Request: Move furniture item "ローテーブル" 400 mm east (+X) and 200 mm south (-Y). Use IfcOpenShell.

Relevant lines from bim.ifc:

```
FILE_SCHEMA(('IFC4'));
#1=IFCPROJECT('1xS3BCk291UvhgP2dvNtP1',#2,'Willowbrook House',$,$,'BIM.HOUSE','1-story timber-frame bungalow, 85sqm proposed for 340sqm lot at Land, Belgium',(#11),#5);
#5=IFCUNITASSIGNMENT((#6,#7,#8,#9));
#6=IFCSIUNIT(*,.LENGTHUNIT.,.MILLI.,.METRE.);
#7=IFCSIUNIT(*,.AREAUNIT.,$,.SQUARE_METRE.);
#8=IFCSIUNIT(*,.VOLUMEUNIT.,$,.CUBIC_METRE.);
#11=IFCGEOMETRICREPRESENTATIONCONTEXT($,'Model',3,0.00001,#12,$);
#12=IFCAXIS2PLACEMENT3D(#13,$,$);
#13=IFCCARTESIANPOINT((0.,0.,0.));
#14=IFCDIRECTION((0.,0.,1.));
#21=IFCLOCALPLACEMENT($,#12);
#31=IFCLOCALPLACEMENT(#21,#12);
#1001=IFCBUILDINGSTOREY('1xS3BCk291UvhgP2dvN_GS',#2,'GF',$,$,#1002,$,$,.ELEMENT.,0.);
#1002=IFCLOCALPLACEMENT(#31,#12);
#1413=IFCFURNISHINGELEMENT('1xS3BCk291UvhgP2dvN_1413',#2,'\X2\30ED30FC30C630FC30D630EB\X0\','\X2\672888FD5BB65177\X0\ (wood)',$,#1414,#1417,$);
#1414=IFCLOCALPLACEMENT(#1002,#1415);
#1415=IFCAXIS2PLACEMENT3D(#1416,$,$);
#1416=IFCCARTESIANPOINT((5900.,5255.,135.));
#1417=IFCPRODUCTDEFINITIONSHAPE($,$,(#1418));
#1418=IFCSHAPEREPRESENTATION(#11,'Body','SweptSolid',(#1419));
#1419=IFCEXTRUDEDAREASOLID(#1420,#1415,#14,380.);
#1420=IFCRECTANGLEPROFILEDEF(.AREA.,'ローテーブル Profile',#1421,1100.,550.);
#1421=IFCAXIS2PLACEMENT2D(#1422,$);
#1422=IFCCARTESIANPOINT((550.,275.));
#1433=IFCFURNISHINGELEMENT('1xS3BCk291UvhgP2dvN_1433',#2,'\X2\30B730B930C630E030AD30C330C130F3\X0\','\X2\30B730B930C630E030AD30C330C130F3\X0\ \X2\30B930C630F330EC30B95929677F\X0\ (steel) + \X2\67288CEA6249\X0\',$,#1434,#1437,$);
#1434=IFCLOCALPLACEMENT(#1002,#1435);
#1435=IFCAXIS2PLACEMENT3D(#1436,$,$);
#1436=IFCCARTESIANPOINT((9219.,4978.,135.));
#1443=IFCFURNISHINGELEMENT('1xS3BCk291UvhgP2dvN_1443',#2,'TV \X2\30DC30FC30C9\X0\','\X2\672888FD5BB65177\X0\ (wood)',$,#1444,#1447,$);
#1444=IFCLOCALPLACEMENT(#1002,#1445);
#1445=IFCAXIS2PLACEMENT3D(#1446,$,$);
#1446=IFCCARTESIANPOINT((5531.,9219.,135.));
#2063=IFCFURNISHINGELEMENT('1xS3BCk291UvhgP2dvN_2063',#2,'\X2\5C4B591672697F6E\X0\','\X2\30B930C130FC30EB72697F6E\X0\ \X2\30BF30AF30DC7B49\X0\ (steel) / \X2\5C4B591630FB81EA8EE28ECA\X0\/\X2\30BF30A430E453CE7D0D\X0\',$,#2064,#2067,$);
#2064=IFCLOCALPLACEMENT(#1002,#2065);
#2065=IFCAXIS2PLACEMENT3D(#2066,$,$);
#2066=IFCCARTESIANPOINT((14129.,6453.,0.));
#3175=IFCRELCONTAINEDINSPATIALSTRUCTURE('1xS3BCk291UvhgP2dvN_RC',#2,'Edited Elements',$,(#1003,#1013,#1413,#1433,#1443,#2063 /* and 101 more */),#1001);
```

```python
import ifcopenshell
import ifcopenshell.api.geometry
import ifcopenshell.util.placement

model = ifcopenshell.open("bim.ifc")

item = model.by_guid("1xS3BCk291UvhgP2dvN_1413")
matrix = ifcopenshell.util.placement.get_local_placement(item.ObjectPlacement)
matrix[0, 3] += 400.0
matrix[1, 3] -= 200.0
ifcopenshell.api.geometry.edit_object_placement(model, product=item, matrix=matrix, is_si=False)

print(ifcopenshell.util.placement.get_local_placement(item.ObjectPlacement).round(3) + 0.0)

model.write("bim_updated.ifc")
```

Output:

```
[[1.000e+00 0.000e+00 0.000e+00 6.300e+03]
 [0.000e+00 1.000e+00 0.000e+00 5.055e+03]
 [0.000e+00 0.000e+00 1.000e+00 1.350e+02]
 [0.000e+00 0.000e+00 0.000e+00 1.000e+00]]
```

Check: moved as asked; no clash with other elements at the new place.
